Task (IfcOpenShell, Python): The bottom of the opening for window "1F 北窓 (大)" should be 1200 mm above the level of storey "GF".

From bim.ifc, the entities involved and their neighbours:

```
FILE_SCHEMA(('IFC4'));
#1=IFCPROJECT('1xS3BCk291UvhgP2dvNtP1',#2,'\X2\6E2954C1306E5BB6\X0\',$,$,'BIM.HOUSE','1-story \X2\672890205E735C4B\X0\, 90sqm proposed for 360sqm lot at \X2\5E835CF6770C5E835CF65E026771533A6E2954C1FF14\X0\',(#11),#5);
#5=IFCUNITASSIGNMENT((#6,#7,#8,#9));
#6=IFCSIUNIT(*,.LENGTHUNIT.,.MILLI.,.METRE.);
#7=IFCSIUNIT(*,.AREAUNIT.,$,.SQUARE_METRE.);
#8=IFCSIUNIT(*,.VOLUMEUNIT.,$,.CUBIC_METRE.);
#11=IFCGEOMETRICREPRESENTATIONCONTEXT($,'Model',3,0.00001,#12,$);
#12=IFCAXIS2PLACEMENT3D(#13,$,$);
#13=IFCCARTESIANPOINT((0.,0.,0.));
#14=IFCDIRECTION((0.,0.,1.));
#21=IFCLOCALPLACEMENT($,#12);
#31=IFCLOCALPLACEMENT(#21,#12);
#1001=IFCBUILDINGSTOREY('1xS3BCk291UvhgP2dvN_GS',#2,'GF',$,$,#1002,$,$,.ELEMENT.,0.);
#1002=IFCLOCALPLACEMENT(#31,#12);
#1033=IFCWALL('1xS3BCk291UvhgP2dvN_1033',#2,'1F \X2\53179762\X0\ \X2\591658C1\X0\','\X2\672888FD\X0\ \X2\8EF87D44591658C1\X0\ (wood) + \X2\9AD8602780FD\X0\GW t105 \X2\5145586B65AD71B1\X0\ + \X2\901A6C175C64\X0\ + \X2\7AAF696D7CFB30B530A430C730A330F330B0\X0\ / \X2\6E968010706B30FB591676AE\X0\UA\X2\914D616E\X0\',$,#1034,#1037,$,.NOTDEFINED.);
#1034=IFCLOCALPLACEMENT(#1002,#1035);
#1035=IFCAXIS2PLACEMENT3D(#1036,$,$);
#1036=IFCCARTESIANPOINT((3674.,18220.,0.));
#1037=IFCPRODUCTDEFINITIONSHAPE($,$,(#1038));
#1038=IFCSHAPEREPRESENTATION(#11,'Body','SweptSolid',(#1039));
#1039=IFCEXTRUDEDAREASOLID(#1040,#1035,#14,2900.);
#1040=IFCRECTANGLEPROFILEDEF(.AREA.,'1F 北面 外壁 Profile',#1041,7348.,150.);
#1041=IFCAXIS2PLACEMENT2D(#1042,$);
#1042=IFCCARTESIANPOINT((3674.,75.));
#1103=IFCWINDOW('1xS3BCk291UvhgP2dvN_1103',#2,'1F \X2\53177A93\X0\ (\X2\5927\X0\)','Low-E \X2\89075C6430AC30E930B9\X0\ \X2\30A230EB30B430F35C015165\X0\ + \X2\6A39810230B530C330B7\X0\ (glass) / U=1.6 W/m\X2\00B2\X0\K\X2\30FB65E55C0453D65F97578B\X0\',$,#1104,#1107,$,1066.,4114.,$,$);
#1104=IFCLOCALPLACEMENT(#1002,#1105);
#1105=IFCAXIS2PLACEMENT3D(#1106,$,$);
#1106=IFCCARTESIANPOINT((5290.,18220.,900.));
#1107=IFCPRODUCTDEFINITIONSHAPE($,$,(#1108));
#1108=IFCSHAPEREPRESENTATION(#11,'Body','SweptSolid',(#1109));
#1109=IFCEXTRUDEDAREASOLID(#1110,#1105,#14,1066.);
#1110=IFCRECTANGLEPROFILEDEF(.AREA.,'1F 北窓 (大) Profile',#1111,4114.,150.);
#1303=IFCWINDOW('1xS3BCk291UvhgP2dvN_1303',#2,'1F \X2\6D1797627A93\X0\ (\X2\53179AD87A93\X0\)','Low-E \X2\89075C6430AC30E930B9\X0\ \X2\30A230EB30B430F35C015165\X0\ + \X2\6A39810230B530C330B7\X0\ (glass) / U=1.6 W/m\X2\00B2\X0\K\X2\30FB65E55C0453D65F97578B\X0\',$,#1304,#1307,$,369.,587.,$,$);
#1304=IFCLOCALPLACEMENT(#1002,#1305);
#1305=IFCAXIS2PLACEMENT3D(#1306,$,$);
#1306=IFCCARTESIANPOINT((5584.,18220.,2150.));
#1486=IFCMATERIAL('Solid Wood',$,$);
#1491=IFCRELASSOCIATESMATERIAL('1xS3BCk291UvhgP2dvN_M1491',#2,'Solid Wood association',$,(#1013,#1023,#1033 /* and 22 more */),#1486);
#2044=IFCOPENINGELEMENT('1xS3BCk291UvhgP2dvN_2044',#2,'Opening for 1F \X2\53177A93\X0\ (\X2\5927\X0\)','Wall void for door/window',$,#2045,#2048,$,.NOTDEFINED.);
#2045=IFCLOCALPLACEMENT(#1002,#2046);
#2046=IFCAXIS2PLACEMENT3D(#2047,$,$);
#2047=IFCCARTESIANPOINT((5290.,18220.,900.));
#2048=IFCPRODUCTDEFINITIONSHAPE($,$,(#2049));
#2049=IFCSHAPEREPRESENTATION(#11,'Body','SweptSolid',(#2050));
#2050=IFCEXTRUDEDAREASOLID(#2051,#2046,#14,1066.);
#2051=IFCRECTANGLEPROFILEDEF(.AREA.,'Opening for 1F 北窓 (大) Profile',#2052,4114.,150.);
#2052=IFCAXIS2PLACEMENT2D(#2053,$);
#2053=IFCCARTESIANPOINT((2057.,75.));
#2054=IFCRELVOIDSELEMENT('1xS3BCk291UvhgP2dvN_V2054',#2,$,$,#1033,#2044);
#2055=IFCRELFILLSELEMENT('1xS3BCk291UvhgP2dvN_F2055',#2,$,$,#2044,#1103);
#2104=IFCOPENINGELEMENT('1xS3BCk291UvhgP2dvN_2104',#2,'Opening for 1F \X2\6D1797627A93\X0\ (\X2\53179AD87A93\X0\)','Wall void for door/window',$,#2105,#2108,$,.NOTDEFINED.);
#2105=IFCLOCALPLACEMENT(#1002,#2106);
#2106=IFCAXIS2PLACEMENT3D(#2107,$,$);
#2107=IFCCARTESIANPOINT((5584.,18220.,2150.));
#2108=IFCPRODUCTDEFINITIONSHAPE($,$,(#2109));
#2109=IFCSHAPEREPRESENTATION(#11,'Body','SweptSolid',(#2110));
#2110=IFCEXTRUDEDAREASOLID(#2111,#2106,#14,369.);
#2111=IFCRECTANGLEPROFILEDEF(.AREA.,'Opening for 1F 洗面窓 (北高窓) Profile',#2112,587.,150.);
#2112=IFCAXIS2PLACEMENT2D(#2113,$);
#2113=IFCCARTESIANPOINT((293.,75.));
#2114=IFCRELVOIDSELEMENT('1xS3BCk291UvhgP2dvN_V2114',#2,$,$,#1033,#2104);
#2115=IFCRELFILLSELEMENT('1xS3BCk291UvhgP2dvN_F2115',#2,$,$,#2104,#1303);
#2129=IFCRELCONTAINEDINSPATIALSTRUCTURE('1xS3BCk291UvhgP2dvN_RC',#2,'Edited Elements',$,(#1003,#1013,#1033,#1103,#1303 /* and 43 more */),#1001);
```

```python
import numpy as np
import ifcopenshell
import ifcopenshell.api.geometry
import ifcopenshell.geom
import ifcopenshell.util.element
import ifcopenshell.util.placement
import ifcopenshell.util.shape
import ifcopenshell.util.unit

model = ifcopenshell.open("bim.ifc")
unit_scale = ifcopenshell.util.unit.calculate_unit_scale(model)

window = model.by_guid("1xS3BCk291UvhgP2dvN_1103")
opening = window.FillsVoids[0].RelatingOpeningElement
storey = ifcopenshell.util.element.get_container(window, ifc_class="IfcBuildingStorey")
level = ifcopenshell.util.placement.get_local_placement(storey.ObjectPlacement)[2, 3]

# The opening's origin need not be at the sill, so measure its lowest point.
shape = ifcopenshell.geom.create_shape(ifcopenshell.geom.settings(), opening)
bottom = ifcopenshell.util.shape.get_shape_bottom_elevation(shape, shape.geometry) / unit_scale
dz = level + 1.2 / unit_scale - bottom

shift = np.array([0.0, 0.0, dz])
# The window is not placed relative to its opening, so move both.
for product in (opening, window):
    matrix = ifcopenshell.util.placement.get_local_placement(product.ObjectPlacement)
    matrix[:3, 3] += shift
    ifcopenshell.api.geometry.edit_object_placement(model, product=product, matrix=matrix, is_si=False)

print(f"moved by {dz * unit_scale:+.3f} m")

model.write("bim_v2.ifc")
```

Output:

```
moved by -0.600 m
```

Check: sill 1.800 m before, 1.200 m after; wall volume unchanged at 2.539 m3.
